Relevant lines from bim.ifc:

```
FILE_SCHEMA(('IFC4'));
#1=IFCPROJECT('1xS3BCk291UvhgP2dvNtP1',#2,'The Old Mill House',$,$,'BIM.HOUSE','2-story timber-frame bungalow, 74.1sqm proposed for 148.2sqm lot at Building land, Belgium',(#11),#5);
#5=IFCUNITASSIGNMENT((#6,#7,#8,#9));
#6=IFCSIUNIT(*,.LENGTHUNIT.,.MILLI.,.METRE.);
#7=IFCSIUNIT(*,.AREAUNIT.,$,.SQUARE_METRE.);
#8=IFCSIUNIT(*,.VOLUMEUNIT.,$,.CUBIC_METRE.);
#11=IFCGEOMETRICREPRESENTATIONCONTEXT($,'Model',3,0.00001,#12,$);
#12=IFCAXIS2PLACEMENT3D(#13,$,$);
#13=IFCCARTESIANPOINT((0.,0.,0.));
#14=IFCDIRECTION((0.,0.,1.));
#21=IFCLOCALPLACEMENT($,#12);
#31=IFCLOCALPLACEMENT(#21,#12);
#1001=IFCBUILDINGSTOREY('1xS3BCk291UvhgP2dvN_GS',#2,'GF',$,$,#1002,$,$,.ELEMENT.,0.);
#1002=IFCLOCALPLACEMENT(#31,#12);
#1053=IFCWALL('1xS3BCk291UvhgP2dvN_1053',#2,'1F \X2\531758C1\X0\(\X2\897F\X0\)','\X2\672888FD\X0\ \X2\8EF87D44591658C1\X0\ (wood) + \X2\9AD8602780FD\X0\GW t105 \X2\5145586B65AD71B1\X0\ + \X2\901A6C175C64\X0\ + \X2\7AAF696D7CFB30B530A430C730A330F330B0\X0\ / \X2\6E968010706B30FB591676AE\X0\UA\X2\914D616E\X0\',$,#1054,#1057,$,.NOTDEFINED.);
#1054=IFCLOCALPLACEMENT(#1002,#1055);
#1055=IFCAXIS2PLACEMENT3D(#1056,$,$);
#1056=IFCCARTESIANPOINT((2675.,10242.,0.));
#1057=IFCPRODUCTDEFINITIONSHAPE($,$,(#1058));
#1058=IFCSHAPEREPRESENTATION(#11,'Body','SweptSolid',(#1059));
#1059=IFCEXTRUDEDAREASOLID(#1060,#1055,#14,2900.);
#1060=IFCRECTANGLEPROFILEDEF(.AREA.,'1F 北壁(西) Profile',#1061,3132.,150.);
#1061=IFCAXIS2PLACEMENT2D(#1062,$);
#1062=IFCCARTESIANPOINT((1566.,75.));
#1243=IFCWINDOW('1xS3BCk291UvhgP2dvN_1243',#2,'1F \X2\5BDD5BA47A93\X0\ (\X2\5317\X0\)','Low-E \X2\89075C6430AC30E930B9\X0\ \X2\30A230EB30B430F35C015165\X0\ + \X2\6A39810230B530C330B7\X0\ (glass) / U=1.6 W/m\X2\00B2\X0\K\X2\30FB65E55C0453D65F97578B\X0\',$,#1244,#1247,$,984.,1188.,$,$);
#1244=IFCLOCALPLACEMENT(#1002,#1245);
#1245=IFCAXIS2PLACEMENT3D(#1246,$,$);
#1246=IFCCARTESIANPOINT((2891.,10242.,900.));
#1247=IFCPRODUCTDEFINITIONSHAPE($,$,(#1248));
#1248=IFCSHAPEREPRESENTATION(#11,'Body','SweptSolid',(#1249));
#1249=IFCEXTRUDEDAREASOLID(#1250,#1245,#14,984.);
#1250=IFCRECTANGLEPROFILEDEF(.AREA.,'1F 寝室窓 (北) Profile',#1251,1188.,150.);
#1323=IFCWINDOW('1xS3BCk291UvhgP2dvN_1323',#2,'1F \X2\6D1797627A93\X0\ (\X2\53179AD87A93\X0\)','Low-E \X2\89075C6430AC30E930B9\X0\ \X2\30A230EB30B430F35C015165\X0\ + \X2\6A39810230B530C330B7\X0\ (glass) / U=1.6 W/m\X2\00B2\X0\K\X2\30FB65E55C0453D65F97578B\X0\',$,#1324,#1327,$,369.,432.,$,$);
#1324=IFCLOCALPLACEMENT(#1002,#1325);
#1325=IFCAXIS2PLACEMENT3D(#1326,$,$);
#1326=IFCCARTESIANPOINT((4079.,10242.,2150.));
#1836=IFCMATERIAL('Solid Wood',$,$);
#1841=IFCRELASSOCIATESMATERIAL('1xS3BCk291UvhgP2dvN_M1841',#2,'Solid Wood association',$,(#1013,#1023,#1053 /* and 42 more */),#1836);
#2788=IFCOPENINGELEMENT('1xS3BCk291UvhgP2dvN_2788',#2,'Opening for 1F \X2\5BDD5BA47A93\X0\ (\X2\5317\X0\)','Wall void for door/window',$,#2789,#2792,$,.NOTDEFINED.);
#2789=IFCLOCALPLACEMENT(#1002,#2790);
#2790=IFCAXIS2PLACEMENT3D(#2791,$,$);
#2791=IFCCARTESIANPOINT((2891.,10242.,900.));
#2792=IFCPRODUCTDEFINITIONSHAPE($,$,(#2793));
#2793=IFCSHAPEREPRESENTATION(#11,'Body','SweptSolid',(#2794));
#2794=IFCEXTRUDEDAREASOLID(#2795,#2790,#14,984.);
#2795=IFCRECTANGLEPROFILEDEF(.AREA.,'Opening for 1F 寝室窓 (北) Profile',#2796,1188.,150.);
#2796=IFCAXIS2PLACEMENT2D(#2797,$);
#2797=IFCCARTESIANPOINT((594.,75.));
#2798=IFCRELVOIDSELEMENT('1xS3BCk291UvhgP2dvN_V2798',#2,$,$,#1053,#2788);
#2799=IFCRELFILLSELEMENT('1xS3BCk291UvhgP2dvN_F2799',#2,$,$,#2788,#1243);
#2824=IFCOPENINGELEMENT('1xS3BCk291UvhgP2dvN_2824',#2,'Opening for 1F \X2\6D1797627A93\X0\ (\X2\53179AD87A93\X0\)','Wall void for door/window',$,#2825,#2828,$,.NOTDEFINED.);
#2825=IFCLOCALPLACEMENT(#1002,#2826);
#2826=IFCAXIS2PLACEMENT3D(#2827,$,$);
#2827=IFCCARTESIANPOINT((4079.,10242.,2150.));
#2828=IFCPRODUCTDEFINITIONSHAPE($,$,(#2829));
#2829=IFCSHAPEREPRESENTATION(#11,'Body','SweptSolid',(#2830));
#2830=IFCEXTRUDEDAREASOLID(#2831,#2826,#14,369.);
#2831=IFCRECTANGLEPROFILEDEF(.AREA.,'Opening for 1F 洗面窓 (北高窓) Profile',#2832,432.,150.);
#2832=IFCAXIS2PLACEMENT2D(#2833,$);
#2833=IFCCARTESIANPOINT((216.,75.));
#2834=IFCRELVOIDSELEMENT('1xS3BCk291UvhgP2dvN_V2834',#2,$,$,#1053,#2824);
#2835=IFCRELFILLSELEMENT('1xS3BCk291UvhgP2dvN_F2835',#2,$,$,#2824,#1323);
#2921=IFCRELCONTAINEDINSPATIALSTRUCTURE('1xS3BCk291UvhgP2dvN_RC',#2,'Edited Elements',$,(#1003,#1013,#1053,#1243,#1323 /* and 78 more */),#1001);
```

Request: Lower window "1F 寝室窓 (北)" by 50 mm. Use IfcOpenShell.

```python
import numpy as np
import ifcopenshell
import ifcopenshell.api.geometry
import ifcopenshell.util.placement
import ifcopenshell.util.unit

model = ifcopenshell.open("bim.ifc")
unit_scale = ifcopenshell.util.unit.calculate_unit_scale(model)

window = model.by_guid("1xS3BCk291UvhgP2dvN_1243")
opening = window.FillsVoids[0].RelatingOpeningElement
dz = -50.0

shift = np.array([0.0, 0.0, dz])
# The window is not placed relative to its opening, so move both.
for product in (opening, window):
    matrix = ifcopenshell.util.placement.get_local_placement(product.ObjectPlacement)
    matrix[:3, 3] += shift
    ifcopenshell.api.geometry.edit_object_placement(model, product=product, matrix=matrix, is_si=False)

print(f"moved by {dz * unit_scale:+.3f} m")

model.write("bim-out.ifc")
```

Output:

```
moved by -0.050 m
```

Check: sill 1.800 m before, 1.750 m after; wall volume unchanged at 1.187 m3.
